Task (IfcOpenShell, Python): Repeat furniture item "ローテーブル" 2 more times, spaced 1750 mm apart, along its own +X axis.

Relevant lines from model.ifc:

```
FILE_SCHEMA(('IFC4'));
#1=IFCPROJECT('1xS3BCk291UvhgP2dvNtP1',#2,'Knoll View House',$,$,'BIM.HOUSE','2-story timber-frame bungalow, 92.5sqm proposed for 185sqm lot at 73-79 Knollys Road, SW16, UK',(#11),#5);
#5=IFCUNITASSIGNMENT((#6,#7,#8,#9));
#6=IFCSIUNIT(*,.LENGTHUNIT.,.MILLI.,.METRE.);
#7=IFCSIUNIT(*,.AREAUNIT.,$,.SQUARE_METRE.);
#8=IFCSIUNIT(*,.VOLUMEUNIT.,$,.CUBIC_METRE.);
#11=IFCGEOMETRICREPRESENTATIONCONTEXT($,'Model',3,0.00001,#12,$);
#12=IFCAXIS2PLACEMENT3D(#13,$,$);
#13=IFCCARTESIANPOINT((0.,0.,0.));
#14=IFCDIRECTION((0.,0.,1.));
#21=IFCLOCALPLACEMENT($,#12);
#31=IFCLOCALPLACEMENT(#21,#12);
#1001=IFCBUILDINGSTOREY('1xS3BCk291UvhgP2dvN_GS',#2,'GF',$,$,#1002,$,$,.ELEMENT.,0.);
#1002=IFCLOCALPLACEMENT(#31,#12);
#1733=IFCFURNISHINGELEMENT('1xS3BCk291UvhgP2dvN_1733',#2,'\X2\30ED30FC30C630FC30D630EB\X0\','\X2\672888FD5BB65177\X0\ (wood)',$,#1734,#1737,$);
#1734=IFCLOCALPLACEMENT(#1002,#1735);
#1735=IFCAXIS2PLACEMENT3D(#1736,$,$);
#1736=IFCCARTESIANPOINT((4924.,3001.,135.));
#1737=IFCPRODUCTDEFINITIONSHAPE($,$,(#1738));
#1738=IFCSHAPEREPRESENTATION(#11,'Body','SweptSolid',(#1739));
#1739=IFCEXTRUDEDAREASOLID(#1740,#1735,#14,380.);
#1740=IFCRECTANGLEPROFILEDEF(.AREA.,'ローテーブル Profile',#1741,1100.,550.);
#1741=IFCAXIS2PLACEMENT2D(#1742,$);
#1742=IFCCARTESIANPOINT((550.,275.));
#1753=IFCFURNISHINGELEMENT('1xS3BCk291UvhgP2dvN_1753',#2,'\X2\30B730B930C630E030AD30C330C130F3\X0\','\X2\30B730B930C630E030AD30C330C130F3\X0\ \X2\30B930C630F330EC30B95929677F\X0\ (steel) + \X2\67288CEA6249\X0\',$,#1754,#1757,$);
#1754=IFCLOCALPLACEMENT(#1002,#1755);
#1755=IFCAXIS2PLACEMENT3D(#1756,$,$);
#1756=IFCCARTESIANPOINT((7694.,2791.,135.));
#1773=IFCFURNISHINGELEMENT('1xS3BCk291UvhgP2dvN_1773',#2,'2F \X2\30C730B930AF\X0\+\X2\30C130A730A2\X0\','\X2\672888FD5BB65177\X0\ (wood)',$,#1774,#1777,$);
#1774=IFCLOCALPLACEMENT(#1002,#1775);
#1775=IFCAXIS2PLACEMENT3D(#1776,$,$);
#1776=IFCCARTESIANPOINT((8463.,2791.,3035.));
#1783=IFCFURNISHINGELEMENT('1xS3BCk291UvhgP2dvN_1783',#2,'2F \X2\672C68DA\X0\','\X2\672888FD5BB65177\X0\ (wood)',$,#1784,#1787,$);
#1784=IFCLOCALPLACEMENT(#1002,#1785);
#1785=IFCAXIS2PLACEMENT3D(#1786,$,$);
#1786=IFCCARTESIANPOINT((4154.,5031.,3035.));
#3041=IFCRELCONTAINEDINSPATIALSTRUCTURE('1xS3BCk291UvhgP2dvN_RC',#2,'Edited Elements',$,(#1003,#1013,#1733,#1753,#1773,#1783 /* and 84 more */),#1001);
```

```python
import ifcopenshell
import ifcopenshell.api.geometry
import ifcopenshell.api.root
import ifcopenshell.util.element
import ifcopenshell.util.placement
import ifcopenshell.util.unit

model = ifcopenshell.open("model.ifc")
unit_scale = ifcopenshell.util.unit.calculate_unit_scale(model)


def reuse_history(source, copy):
    """copy_class also copies each property set's owner history, people and application; keep the originals."""
    for rel in copy.IsDefinedBy:
        if rel.is_a("IfcRelDefinesByProperties") and (history := rel.RelatingPropertyDefinition.OwnerHistory):
            rel.RelatingPropertyDefinition.OwnerHistory = source.OwnerHistory
            ifcopenshell.util.element.remove_deep2(model, history)


source = model.by_guid("1xS3BCk291UvhgP2dvN_1733")
base = ifcopenshell.util.placement.get_local_placement(source.ObjectPlacement)
step = base[:3, 0] * 1.75 / unit_scale

for i in range(1, 3):
    copy = ifcopenshell.api.root.copy_class(model, product=source)
    copy.Representation = ifcopenshell.util.element.copy_deep(
        model, source.Representation, exclude=["IfcGeometricRepresentationContext", "IfcRepresentationMap"]
    )
    reuse_history(source, copy)
    matrix = base.copy()
    matrix[:3, 3] += i * step
    print("added at", matrix[:3, 3].round(3) + 0.0)
    ifcopenshell.api.geometry.edit_object_placement(model, product=copy, matrix=matrix, is_si=False)

model.write("model_rev.ifc")
```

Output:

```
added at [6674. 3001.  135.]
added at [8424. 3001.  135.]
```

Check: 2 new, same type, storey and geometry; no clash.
